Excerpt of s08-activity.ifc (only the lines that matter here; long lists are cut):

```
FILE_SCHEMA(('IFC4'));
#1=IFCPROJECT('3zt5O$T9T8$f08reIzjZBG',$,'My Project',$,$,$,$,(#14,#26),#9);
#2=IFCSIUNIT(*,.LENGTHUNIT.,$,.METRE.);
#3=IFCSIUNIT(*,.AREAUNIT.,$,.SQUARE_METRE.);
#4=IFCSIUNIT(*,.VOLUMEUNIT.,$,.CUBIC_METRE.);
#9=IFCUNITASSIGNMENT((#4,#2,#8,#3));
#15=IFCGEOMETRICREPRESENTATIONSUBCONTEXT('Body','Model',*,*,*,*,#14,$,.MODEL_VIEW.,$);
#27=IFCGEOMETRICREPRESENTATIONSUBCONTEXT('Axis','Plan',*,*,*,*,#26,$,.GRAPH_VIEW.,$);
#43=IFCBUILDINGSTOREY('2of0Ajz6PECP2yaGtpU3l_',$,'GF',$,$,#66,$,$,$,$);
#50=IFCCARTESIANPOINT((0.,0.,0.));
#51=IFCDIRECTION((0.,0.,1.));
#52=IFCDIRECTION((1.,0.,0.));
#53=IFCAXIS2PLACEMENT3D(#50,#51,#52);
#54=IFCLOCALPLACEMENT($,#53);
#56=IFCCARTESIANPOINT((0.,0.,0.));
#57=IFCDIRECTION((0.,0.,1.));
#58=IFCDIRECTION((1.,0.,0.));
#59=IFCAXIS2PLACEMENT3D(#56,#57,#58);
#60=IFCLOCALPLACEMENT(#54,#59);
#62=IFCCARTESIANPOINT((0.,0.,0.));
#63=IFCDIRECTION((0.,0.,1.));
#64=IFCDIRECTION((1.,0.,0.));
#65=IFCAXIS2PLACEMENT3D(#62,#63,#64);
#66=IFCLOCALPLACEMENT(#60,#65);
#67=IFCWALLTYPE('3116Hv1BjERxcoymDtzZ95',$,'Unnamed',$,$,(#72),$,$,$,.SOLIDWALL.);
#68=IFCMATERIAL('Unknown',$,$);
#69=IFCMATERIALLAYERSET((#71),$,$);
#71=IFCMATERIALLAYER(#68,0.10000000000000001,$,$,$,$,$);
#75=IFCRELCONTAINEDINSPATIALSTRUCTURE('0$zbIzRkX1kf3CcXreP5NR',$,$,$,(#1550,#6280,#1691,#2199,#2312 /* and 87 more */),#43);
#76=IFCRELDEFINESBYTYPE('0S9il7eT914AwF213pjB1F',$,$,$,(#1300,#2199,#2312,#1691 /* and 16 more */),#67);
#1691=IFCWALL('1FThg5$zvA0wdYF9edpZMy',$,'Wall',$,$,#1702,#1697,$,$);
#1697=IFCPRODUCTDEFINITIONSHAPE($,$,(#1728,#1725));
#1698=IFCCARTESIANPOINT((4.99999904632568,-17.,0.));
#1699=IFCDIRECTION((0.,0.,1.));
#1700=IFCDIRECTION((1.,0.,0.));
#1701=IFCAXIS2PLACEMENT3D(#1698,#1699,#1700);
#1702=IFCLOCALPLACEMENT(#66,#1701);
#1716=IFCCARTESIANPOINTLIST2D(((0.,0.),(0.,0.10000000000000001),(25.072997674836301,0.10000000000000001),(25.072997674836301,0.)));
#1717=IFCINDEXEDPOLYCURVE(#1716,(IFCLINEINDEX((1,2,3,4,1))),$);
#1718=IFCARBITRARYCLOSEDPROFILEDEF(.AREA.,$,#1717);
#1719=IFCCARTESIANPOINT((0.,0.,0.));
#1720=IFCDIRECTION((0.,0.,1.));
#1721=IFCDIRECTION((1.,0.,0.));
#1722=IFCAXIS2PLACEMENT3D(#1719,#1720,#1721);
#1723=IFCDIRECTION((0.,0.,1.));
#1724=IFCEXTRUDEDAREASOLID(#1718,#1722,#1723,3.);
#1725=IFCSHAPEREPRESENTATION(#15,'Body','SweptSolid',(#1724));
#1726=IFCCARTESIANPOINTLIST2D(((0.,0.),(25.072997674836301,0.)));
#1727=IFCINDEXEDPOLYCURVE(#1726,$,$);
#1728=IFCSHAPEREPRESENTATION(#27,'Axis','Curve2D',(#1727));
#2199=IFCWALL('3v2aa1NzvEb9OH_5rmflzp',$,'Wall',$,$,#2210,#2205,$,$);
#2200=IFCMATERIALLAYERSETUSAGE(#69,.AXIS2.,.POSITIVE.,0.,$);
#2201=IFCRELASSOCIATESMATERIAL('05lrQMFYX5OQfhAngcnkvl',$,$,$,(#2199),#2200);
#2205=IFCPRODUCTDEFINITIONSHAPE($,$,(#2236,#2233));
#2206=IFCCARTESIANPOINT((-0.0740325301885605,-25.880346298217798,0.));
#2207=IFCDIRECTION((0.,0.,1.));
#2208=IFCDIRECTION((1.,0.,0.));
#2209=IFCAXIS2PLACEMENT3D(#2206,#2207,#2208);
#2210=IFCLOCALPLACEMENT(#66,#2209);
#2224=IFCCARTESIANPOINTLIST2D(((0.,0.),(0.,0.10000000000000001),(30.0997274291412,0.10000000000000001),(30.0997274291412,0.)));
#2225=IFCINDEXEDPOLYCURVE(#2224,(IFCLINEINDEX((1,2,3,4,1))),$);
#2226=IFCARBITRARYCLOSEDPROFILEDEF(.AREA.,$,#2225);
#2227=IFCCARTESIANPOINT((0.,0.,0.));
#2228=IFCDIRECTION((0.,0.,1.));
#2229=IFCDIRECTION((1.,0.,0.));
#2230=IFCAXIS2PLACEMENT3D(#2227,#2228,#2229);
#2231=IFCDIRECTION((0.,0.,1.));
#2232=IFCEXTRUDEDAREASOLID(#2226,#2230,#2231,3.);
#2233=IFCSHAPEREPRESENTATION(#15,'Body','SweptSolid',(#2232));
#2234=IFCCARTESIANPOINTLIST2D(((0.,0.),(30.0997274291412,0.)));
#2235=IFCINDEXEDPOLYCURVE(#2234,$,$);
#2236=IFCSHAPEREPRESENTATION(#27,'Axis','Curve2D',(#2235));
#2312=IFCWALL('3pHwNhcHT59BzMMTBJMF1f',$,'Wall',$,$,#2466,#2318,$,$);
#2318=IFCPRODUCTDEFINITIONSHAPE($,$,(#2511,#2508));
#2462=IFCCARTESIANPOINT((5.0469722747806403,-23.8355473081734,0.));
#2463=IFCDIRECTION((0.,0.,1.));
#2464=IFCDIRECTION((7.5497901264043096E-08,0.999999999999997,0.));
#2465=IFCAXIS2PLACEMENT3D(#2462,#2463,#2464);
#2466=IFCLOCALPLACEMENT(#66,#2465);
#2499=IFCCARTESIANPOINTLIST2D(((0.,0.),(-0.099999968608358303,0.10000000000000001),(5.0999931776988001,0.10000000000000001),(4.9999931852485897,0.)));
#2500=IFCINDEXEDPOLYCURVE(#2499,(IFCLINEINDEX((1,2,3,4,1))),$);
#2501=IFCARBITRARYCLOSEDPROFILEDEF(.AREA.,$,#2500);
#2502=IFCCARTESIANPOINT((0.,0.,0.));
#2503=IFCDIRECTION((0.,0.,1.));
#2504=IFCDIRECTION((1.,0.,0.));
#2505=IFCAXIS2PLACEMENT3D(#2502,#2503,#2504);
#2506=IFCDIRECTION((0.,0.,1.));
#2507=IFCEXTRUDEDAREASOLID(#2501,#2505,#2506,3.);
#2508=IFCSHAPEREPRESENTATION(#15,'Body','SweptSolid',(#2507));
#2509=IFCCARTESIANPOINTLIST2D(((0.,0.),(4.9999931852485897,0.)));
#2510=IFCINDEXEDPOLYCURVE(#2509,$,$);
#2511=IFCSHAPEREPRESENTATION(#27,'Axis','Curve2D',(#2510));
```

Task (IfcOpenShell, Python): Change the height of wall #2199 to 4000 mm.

```python
import ifcopenshell
import ifcopenshell.geom
import ifcopenshell.util.representation
import ifcopenshell.util.shape

model = ifcopenshell.open("s08-activity.ifc")
settings = ifcopenshell.geom.settings()


def volume(element):
    """Net volume in cubic metres, openings subtracted."""
    shape = ifcopenshell.geom.create_shape(settings, element)
    return ifcopenshell.util.shape.get_volume(shape.geometry)


wall = model.by_guid("3v2aa1NzvEb9OH_5rmflzp")
before = volume(wall)

body = ifcopenshell.util.representation.get_representation(wall, "Model", "Body")
solid = body.Items[0]
old_height = solid.Depth
solid.Depth = 4.0
after = volume(wall)

print(f"height {old_height:g} -> {solid.Depth:g}, volume {before:.3f} -> {after:.3f} m3")

model.write("s08-activity_edited.ifc")
```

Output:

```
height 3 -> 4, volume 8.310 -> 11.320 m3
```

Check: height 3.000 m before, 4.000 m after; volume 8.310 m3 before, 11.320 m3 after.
